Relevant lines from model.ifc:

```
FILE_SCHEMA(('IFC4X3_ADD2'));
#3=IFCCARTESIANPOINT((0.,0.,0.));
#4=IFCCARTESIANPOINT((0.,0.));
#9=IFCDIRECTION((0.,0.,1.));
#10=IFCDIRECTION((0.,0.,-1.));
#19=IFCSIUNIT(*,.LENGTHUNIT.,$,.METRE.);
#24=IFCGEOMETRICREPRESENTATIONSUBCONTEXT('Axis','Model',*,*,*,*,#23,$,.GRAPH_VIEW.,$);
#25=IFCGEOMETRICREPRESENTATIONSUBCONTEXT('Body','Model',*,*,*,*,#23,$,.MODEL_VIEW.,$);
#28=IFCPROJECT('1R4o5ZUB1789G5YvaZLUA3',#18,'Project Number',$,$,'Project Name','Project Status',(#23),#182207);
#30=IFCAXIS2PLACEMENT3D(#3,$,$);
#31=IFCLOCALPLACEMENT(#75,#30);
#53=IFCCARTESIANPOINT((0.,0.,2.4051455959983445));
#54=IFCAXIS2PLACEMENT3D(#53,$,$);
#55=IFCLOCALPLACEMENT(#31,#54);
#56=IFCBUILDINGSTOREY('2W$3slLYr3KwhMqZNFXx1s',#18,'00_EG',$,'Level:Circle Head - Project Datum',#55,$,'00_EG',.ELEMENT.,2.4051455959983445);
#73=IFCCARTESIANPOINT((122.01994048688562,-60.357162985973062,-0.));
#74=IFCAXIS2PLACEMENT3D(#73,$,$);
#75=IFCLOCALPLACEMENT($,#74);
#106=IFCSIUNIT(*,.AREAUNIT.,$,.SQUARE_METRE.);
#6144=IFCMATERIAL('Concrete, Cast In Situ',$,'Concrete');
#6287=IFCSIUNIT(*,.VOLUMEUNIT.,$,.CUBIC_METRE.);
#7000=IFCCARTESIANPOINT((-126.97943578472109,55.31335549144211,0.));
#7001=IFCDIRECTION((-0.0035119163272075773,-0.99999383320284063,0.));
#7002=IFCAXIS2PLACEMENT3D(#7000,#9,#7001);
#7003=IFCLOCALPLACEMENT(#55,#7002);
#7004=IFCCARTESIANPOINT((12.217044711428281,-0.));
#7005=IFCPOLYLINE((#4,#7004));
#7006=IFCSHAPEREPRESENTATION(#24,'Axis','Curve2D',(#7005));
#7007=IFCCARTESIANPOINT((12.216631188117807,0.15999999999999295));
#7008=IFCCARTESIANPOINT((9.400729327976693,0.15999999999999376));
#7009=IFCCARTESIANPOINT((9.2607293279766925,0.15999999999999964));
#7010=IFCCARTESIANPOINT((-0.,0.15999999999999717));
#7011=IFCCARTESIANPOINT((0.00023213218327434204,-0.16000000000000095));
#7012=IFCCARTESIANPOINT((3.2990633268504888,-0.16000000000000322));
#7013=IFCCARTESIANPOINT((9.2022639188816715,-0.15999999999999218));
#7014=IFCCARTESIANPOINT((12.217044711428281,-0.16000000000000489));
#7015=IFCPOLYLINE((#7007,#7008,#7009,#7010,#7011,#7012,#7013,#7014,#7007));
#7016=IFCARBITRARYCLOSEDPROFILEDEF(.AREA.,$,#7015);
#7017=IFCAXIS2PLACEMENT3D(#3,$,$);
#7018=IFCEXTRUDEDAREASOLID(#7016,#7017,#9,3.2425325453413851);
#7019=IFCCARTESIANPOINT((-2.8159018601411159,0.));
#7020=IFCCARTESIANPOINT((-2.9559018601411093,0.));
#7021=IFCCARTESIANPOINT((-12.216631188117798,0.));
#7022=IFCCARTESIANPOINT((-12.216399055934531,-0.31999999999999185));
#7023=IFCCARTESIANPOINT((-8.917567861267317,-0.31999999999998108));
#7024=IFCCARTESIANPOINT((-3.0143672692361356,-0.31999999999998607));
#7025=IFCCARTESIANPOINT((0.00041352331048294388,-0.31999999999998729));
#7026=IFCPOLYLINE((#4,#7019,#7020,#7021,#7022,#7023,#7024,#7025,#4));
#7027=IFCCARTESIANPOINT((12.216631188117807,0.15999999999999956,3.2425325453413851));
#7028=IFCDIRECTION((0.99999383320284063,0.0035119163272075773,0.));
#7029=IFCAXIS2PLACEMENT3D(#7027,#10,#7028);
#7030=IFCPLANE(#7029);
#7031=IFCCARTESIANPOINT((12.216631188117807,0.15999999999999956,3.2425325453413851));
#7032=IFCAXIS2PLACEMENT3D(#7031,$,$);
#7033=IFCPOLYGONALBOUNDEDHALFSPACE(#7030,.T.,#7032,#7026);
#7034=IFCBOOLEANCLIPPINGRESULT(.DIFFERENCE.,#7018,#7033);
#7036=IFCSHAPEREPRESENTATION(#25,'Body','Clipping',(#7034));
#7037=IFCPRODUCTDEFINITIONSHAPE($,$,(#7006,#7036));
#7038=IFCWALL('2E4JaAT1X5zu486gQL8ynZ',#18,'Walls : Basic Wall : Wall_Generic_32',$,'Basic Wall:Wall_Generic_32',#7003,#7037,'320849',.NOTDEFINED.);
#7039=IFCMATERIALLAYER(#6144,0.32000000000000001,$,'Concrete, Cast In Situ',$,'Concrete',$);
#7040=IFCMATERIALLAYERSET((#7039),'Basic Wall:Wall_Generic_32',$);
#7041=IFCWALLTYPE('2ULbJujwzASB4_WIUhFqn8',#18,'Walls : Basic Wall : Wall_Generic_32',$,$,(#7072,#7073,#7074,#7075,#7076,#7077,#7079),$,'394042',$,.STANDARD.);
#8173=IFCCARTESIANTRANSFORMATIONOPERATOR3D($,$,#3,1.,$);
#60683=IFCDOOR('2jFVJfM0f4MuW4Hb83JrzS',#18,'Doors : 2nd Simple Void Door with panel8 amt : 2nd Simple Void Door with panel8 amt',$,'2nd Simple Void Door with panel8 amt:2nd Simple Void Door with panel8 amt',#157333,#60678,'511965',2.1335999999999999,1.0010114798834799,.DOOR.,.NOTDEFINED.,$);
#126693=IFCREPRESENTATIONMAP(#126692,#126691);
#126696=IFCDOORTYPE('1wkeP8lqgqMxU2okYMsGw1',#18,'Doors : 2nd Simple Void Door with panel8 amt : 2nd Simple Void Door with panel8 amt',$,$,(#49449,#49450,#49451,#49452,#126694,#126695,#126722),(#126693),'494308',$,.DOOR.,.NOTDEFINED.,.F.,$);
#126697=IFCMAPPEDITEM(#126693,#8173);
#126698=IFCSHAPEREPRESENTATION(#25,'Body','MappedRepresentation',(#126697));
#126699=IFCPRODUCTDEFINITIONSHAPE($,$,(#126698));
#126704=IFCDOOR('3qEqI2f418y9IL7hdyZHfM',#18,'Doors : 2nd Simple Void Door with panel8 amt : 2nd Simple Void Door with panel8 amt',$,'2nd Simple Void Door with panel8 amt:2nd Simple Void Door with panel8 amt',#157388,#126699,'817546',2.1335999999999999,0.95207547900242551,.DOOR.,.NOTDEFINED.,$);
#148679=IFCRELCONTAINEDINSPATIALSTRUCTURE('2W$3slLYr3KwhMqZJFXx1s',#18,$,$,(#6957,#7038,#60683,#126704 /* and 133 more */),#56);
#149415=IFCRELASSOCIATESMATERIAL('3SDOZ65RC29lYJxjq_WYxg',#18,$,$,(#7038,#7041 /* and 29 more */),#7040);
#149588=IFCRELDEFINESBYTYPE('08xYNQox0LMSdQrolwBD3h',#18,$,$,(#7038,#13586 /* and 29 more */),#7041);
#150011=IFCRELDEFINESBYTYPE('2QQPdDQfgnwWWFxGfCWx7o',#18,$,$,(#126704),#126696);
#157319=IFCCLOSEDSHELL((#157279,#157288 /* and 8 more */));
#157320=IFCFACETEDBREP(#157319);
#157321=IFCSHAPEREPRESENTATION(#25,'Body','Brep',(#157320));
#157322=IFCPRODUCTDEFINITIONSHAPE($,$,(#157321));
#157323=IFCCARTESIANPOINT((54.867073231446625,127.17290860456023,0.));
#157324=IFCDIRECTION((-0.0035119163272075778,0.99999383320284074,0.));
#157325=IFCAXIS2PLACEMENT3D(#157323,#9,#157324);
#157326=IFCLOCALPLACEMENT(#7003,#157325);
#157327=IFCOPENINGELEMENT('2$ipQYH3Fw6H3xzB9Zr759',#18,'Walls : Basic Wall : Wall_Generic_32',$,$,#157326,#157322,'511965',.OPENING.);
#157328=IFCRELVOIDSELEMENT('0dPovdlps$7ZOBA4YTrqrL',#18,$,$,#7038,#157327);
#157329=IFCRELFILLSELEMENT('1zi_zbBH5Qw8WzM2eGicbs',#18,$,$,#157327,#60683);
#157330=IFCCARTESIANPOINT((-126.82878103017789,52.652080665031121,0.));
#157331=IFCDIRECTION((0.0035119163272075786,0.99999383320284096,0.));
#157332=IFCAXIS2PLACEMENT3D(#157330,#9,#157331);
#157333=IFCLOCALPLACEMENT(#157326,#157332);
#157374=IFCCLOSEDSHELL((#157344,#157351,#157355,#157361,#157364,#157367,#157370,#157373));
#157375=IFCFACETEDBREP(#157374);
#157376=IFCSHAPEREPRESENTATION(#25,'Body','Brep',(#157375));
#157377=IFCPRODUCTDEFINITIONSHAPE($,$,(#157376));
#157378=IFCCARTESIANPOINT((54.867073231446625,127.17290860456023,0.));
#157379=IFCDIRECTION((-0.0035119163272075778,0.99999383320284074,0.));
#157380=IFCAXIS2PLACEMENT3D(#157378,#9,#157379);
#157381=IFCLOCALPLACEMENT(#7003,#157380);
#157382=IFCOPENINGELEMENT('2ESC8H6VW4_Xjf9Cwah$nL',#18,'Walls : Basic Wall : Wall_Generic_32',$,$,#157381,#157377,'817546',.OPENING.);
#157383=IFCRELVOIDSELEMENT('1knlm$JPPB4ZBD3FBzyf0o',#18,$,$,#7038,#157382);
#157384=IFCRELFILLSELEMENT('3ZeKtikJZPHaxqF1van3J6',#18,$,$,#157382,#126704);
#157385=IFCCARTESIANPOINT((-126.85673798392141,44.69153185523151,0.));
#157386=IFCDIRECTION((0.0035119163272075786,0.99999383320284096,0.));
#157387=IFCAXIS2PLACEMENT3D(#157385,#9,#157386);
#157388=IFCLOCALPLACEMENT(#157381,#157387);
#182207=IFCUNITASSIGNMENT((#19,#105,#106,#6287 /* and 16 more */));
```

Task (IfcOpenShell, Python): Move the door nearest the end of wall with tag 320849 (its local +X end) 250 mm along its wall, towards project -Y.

```python
import ifcopenshell
import ifcopenshell.api.geometry
import ifcopenshell.util.placement

model = ifcopenshell.open("model.ifc")

door = model.by_guid("3qEqI2f418y9IL7hdyZHfM")
opening = door.FillsVoids[0].RelatingOpeningElement
wall = opening.VoidsElements[0].RelatingBuildingElement

wall_matrix = ifcopenshell.util.placement.get_local_placement(wall.ObjectPlacement)
shift = wall_matrix[:3, 0] * 0.25
before = ifcopenshell.util.placement.get_local_placement(door.ObjectPlacement)[:3, 3].copy()

# The door is placed relative to its opening, so it follows when the opening moves.
matrix = ifcopenshell.util.placement.get_local_placement(opening.ObjectPlacement)
matrix[:3, 3] += shift
ifcopenshell.api.geometry.edit_object_placement(
    model, product=opening, matrix=matrix, is_si=False, should_transform_children=True
)

after = ifcopenshell.util.placement.get_local_placement(door.ObjectPlacement)[:3, 3]
print("door moved by", (after - before).round(3) + 0.0)

model.write("model_v2.ifc")
```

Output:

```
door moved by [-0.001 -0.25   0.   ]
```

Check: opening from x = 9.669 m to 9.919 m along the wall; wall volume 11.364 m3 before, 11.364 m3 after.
